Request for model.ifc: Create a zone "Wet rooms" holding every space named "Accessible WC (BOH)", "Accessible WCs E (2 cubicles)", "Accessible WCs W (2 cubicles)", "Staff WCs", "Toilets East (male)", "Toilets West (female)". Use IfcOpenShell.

First a look at what the model holds.

```python
import ifcopenshell

model = ifcopenshell.open("model.ifc")
print(model.schema)
seen = {}
for space in model.by_type("IfcSpace"):
    seen[space.LongName] = seen.get(space.LongName, 0) + 1
for name, count in sorted(seen.items(), key=str):
    print(count, "x", name)
print("zones:", [z.Name for z in model.by_type("IfcZone")][:20])
```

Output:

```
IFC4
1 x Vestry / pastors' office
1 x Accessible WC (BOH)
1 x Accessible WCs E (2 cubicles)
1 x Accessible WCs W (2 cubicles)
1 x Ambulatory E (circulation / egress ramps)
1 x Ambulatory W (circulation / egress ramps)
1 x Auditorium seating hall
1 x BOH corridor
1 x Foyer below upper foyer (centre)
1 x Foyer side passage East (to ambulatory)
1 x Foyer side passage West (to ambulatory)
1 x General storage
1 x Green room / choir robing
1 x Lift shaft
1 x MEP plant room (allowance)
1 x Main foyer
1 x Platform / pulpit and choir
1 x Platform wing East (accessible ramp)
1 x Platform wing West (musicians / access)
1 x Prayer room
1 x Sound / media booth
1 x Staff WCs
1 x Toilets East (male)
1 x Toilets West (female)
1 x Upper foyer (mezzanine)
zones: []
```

```python
import ifcopenshell
import ifcopenshell.api.group
import ifcopenshell.api.root

model = ifcopenshell.open("model.ifc")

names = {"Accessible WC (BOH)", "Accessible WCs E (2 cubicles)", "Accessible WCs W (2 cubicles)", "Staff WCs", "Toilets East (male)", "Toilets West (female)"}
spaces = [s for s in model.by_type("IfcSpace") if s.LongName in names]

zone = ifcopenshell.api.root.create_entity(model, ifc_class="IfcZone", name="Wet rooms")
ifcopenshell.api.group.assign_group(model, products=spaces, group=zone)
print(len(spaces), "spaces in", zone.Name)

model.write("model_updated.ifc")
```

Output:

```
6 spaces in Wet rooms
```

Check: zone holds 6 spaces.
